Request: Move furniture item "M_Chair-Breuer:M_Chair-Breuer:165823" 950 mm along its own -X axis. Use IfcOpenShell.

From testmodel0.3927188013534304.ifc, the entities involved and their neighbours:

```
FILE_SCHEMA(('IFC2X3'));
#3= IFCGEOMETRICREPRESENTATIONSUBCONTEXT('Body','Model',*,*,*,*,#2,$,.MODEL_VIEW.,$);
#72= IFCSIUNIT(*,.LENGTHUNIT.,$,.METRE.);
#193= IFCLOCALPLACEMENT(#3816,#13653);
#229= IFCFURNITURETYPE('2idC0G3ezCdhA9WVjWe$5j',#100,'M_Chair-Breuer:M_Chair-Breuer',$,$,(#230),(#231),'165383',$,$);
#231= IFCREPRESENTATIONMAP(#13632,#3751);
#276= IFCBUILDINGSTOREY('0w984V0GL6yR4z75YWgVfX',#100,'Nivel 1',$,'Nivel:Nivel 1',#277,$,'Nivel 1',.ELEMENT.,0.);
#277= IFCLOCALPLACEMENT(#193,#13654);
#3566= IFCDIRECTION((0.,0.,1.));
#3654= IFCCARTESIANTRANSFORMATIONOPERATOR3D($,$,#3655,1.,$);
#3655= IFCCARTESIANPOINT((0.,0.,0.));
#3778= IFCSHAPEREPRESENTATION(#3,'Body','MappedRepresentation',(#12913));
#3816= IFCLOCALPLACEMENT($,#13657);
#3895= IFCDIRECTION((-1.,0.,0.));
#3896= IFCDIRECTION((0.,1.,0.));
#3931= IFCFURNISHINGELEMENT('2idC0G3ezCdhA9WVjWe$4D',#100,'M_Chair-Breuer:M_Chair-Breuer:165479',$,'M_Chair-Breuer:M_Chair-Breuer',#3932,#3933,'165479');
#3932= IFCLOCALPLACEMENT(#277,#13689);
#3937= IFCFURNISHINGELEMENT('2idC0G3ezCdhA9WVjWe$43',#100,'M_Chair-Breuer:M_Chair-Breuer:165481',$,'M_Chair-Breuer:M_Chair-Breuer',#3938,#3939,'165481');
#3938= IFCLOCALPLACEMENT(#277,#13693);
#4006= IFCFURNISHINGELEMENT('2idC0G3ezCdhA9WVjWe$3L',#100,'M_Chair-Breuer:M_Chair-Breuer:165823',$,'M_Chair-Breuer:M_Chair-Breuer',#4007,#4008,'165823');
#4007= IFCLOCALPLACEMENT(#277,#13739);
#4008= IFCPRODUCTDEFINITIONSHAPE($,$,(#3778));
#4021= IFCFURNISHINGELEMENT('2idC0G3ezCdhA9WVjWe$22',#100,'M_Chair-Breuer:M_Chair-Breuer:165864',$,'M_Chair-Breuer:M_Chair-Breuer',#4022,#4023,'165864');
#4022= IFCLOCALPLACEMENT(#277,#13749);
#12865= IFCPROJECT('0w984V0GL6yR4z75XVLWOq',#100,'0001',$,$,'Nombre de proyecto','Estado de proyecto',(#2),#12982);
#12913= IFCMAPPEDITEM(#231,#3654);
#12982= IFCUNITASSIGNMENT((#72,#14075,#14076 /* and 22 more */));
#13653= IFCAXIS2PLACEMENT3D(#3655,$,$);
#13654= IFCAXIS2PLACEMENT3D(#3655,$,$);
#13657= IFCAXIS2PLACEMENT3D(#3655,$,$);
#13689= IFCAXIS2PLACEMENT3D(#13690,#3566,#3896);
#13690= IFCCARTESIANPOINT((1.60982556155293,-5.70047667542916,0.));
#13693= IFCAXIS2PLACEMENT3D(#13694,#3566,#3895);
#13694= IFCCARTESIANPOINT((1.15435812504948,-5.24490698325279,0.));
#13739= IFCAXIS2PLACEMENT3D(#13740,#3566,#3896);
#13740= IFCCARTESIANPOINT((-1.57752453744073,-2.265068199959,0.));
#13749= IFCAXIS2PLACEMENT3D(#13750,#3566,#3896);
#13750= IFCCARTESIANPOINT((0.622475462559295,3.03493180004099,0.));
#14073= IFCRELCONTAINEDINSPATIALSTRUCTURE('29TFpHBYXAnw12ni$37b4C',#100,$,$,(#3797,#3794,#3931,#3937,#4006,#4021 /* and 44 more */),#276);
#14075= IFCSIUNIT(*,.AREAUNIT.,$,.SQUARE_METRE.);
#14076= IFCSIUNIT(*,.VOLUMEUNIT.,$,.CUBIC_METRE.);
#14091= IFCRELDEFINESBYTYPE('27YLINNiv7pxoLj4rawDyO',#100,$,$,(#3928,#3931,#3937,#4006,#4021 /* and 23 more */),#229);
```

```python
import ifcopenshell
import ifcopenshell.api.geometry
import ifcopenshell.util.placement

model = ifcopenshell.open("testmodel0.3927188013534304.ifc")

item = model.by_guid("2idC0G3ezCdhA9WVjWe$3L")
matrix = ifcopenshell.util.placement.get_local_placement(item.ObjectPlacement)
matrix[:3, 3] -= matrix[:3, 0] * 0.95
ifcopenshell.api.geometry.edit_object_placement(model, product=item, matrix=matrix, is_si=False)

print(ifcopenshell.util.placement.get_local_placement(item.ObjectPlacement).round(3) + 0.0)

model.write("testmodel0.3927188013534304_edited.ifc")
```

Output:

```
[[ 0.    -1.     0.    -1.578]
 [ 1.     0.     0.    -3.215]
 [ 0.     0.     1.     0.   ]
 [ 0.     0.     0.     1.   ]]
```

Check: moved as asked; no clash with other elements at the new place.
